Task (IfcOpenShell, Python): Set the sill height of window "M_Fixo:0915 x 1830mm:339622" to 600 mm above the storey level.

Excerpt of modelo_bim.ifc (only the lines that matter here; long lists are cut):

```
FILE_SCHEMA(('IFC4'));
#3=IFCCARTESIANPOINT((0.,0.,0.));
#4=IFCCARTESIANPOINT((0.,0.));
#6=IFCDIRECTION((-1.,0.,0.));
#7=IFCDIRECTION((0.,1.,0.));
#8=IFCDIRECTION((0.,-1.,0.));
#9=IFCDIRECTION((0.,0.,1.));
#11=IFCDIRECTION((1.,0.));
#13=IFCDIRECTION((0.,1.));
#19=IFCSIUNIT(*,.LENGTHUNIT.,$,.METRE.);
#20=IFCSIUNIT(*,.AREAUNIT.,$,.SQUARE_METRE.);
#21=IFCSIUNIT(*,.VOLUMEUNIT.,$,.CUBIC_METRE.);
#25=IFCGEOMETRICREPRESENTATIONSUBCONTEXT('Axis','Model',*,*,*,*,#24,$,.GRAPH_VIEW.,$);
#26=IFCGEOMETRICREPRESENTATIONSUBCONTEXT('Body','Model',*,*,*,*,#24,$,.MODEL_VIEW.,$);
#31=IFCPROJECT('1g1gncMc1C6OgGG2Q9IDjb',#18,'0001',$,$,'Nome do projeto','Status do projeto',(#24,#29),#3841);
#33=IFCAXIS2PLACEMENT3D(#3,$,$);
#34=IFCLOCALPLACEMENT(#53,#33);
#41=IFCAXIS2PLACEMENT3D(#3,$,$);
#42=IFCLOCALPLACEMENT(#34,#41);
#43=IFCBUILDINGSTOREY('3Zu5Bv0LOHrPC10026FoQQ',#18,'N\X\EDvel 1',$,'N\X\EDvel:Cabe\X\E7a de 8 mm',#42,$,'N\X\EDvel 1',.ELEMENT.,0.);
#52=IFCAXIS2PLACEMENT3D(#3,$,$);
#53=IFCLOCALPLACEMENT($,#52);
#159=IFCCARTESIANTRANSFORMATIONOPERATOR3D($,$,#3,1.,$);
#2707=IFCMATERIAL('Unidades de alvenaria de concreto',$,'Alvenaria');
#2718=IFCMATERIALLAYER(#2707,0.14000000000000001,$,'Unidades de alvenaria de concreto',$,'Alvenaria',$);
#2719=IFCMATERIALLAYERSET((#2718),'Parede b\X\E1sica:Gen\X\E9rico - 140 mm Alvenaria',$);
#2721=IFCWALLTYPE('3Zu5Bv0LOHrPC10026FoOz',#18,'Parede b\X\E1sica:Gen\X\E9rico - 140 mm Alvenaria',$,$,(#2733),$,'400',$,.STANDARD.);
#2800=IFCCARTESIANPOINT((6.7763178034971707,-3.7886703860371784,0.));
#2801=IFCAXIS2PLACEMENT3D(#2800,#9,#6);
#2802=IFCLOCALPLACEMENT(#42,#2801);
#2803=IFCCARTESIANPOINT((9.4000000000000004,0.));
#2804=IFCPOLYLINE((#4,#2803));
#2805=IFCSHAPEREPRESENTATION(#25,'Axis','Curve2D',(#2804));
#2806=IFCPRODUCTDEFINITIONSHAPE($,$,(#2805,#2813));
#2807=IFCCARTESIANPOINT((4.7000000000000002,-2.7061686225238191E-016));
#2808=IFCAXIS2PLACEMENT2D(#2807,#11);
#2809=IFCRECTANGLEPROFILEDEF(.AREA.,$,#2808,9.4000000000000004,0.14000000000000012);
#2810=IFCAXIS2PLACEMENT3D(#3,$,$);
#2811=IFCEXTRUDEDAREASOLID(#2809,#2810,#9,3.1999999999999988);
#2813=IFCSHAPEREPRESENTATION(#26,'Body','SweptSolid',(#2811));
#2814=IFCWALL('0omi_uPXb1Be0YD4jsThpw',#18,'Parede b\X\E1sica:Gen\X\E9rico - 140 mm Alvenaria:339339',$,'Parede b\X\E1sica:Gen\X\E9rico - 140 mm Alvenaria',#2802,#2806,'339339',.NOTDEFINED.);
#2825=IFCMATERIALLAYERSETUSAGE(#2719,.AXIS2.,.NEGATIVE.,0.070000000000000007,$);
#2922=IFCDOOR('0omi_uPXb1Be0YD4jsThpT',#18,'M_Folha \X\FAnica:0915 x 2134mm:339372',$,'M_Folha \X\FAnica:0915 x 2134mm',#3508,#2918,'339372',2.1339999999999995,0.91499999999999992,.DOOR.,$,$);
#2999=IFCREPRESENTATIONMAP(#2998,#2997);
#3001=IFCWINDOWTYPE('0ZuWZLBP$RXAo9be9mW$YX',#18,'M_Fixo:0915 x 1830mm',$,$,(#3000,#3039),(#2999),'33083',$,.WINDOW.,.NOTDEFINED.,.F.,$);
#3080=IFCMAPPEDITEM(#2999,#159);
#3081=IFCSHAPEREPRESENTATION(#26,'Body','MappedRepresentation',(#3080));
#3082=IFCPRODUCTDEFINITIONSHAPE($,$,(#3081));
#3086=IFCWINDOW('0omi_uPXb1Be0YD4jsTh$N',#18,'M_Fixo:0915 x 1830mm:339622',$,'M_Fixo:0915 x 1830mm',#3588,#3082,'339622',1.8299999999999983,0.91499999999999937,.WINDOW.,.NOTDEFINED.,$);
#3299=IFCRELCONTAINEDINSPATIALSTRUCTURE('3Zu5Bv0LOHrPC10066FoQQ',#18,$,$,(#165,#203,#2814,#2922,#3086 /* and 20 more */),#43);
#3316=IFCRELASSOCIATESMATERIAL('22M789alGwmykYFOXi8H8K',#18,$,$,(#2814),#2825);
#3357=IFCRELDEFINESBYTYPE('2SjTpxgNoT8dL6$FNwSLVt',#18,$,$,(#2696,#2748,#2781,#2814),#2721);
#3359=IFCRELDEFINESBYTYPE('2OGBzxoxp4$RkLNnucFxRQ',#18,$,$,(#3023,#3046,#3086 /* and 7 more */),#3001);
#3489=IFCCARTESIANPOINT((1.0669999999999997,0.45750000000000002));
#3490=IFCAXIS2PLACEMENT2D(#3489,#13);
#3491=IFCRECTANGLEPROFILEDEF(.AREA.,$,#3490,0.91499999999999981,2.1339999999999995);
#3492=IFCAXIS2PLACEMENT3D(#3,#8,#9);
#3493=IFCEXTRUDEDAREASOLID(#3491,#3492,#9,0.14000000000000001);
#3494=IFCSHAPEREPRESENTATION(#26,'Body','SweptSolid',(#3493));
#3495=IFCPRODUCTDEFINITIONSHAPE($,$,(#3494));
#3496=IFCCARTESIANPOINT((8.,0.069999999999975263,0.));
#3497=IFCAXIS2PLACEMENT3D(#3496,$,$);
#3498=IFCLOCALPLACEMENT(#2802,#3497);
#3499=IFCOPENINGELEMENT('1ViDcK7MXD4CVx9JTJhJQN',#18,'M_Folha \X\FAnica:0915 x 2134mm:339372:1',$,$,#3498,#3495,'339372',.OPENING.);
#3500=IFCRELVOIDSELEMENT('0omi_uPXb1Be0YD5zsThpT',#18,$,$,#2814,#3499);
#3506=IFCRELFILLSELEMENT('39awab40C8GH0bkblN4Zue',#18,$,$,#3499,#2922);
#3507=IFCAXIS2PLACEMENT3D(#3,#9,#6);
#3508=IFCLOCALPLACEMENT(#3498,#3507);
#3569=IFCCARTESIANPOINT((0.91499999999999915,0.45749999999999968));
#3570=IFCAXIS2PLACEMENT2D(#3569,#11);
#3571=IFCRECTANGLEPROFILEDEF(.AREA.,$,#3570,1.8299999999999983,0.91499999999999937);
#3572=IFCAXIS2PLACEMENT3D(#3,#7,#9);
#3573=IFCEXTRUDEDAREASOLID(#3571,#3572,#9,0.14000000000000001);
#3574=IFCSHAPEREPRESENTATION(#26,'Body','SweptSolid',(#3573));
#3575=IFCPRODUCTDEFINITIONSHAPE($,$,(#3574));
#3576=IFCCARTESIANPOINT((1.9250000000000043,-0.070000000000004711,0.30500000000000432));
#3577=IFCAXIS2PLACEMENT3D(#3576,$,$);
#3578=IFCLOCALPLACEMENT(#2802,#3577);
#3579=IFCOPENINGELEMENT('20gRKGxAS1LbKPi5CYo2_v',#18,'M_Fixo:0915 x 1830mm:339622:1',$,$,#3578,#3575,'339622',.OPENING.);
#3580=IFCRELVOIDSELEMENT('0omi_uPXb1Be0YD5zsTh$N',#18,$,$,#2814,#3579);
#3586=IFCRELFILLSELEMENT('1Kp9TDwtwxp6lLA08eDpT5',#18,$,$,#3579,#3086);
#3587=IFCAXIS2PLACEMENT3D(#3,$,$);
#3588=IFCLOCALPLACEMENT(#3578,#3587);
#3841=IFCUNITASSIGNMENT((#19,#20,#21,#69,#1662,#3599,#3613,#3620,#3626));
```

```python
import numpy as np
import ifcopenshell
import ifcopenshell.api.geometry
import ifcopenshell.geom
import ifcopenshell.util.element
import ifcopenshell.util.placement
import ifcopenshell.util.shape
import ifcopenshell.util.unit

model = ifcopenshell.open("modelo_bim.ifc")
unit_scale = ifcopenshell.util.unit.calculate_unit_scale(model)

window = model.by_id(3086)
opening = window.FillsVoids[0].RelatingOpeningElement
storey = ifcopenshell.util.element.get_container(window, ifc_class="IfcBuildingStorey")
level = ifcopenshell.util.placement.get_local_placement(storey.ObjectPlacement)[2, 3]

# The opening's origin need not be at the sill, so measure its lowest point.
shape = ifcopenshell.geom.create_shape(ifcopenshell.geom.settings(), opening)
bottom = ifcopenshell.util.shape.get_shape_bottom_elevation(shape, shape.geometry) / unit_scale
dz = level + 0.6 - bottom

shift = np.array([0.0, 0.0, dz])
# The window is placed relative to its opening, so it follows when the opening moves.
matrix = ifcopenshell.util.placement.get_local_placement(opening.ObjectPlacement)
matrix[:3, 3] += shift
ifcopenshell.api.geometry.edit_object_placement(
    model, product=opening, matrix=matrix, is_si=False, should_transform_children=True
)

print(f"moved by {dz * unit_scale:+.3f} m")

model.write("modelo_bim_v2.ifc")
```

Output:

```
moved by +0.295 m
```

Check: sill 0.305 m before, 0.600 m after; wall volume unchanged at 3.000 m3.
